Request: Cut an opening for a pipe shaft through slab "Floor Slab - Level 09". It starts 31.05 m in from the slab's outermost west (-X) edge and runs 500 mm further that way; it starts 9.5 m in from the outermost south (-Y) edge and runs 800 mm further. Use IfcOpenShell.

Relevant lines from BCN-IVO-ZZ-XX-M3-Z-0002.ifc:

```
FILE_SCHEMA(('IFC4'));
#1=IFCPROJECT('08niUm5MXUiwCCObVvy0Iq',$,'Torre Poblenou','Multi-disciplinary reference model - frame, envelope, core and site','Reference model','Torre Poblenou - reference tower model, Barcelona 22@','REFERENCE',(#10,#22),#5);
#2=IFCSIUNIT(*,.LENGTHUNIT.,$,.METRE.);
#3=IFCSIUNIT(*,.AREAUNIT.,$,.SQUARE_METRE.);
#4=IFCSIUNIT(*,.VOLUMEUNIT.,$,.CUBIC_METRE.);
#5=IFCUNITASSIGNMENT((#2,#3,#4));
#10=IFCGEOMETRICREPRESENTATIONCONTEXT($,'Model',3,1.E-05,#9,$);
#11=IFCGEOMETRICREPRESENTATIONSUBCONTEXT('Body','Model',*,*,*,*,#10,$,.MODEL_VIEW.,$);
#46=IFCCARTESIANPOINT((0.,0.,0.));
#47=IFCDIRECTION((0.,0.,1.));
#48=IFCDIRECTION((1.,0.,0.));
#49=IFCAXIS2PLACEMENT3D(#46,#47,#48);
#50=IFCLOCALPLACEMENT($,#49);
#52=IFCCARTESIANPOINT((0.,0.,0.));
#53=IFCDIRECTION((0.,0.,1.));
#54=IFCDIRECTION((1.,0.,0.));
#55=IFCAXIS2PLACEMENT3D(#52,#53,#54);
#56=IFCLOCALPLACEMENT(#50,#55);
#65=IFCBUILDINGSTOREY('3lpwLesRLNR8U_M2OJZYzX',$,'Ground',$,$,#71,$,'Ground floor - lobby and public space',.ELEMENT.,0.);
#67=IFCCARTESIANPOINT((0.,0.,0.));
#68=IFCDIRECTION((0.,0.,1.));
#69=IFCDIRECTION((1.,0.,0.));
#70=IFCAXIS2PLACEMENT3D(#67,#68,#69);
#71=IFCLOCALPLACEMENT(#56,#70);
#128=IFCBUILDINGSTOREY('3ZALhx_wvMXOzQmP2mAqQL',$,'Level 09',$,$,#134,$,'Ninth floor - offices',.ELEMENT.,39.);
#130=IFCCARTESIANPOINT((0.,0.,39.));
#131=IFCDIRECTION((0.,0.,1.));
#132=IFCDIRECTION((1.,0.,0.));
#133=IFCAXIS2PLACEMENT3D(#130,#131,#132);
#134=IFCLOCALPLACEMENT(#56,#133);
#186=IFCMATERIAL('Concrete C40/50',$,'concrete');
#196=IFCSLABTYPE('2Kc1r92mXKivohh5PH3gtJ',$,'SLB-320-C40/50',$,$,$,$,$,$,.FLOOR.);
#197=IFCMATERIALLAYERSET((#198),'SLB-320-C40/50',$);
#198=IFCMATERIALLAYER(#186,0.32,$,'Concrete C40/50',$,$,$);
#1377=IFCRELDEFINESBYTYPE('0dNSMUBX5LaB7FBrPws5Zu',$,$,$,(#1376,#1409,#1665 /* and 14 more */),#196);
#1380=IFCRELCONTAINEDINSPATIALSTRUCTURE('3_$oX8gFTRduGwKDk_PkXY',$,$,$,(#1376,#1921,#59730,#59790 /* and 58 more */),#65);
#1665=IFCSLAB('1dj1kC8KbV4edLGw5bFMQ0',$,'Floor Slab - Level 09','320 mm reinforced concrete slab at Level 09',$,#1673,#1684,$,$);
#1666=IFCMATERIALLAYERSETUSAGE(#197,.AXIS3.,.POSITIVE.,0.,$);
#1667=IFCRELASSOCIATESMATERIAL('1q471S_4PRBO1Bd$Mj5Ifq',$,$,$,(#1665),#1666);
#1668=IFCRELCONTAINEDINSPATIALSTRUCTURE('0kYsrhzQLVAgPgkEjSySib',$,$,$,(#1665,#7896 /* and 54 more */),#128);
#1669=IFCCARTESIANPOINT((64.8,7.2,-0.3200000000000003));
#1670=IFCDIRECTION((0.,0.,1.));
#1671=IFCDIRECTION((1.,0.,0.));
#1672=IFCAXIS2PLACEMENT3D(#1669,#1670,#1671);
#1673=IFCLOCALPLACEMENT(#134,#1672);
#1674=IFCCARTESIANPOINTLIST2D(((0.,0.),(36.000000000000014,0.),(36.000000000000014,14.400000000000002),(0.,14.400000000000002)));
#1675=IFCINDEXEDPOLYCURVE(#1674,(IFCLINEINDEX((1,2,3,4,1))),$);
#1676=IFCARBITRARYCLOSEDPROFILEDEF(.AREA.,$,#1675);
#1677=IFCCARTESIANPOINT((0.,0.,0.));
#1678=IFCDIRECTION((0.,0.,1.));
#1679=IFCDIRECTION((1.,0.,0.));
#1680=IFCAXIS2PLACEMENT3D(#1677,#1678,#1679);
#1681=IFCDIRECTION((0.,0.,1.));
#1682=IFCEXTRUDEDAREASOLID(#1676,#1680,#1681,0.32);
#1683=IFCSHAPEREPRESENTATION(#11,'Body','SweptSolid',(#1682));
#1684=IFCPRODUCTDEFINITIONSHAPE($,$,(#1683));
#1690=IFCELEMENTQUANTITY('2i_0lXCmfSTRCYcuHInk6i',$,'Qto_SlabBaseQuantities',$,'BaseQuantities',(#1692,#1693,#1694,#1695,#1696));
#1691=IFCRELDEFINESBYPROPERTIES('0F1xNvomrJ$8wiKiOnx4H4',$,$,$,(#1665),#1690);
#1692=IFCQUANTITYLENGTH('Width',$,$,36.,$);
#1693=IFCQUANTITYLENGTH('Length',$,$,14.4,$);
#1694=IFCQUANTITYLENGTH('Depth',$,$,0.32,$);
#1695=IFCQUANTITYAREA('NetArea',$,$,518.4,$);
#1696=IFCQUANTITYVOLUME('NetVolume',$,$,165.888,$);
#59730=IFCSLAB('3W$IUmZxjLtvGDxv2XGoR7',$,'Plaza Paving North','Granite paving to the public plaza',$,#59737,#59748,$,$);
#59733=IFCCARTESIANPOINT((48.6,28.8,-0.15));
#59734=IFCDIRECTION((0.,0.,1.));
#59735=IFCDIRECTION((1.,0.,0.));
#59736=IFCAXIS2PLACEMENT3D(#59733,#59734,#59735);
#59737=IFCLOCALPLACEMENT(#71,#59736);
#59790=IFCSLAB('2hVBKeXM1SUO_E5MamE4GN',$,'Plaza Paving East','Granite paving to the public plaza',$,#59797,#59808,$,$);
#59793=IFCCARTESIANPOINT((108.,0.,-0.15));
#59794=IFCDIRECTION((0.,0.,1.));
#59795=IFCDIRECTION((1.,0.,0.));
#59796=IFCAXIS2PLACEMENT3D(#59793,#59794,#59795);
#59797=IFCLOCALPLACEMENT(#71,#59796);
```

```python
import numpy as np
import ifcopenshell
import ifcopenshell.api.feature
import ifcopenshell.api.geometry
import ifcopenshell.api.pset
import ifcopenshell.api.root
import ifcopenshell.geom
import ifcopenshell.util.element
import ifcopenshell.util.placement
import ifcopenshell.util.representation
import ifcopenshell.util.shape
import ifcopenshell.util.unit

model = ifcopenshell.open("BCN-IVO-ZZ-XX-M3-Z-0002.ifc")
unit_scale = ifcopenshell.util.unit.calculate_unit_scale(model)
area_scale = ifcopenshell.util.unit.calculate_unit_scale(model, "AREAUNIT")
volume_scale = ifcopenshell.util.unit.calculate_unit_scale(model, "VOLUMEUNIT")
settings = ifcopenshell.geom.settings()


def volume(element):
    """Net volume in cubic metres, openings subtracted."""
    shape = ifcopenshell.geom.create_shape(settings, element)
    return ifcopenshell.util.shape.get_volume(shape.geometry)


slab = model.by_guid("1dj1kC8KbV4edLGw5bFMQ0")
before = volume(slab)

# Extent in the slab's own axes, in metres. The edges named are its -X and -Y sides.
slab_shape = ifcopenshell.geom.create_shape(settings, slab)
vertices = ifcopenshell.util.shape.get_vertices(slab_shape.geometry)
x_min, y_min, bottom = vertices.min(axis=0)
top = vertices[:, 2].max()

opening = ifcopenshell.api.root.create_entity(model, ifc_class="IfcOpeningElement", name="Pipe shaft opening", predefined_type="OPENING")
context = ifcopenshell.util.representation.get_context(model, "Model", "Body", "MODEL_VIEW")
width, depth = 0.5, 0.8
outline = [(0.0, 0.0), (width, 0.0), (width, depth), (0.0, depth), (0.0, 0.0)]
# Overshoot both faces by 50 mm so the cut is clean.
shape = ifcopenshell.api.geometry.add_slab_representation(
    model, context=context, depth=top - bottom + 0.1, polyline=outline
)
ifcopenshell.api.geometry.assign_representation(model, product=opening, representation=shape)

matrix = ifcopenshell.util.placement.get_local_placement(slab.ObjectPlacement)
matrix[:, 3] = matrix @ np.append(np.array([x_min + 31.05, y_min + 9.5, bottom - 0.05]) / unit_scale, 1.0)
ifcopenshell.api.geometry.edit_object_placement(model, product=opening, matrix=matrix, is_si=False)
ifcopenshell.api.feature.add_feature(model, feature=opening, element=slab)

after = volume(slab)

# Update the slab's stored quantities.
qto = model.by_id(ifcopenshell.util.element.get_pset(slab, "Qto_SlabBaseQuantities", should_inherit=False)["id"])
ifcopenshell.api.pset.edit_qto(model, qto=qto, properties={
    "NetArea": after / (top - bottom) / area_scale,
    "NetVolume": after / volume_scale,
})

print(f"slab volume {before:.3f} -> {after:.3f} m3")

model.write("BCN-IVO-ZZ-XX-M3-Z-0002_updated.ifc")
```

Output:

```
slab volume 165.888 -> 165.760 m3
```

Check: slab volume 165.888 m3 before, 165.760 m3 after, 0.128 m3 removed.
